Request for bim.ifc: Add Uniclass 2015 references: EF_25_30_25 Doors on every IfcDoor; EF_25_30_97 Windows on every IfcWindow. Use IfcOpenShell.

First a look at what the model holds.

```python
import ifcopenshell

model = ifcopenshell.open("bim.ifc")
print(model.schema)
print("classifications:", [c.Name for c in model.by_type("IfcClassification")])
for ifc_class in ("IfcDoor", "IfcRoof", "IfcStair", "IfcWall", "IfcWindow"):
    print(ifc_class, len(model.by_type(ifc_class)))
```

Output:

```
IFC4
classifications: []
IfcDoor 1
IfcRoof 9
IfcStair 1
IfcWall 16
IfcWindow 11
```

```python
import ifcopenshell
import ifcopenshell.api.classification

model = ifcopenshell.open("bim.ifc")

system = ifcopenshell.api.classification.add_classification(model, classification="Uniclass 2015")

codes = {
    "IfcDoor": ("EF_25_30_25", "Doors"),
    "IfcWindow": ("EF_25_30_97", "Windows"),
}
for ifc_class, (code, name) in codes.items():
    products = model.by_type(ifc_class)
    ifcopenshell.api.classification.add_reference(
        model, products=products, classification=system, identification=code, name=name
    )
    print(code, len(products))

model.write("bim_rev.ifc")
```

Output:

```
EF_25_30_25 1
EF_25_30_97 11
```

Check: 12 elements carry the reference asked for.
